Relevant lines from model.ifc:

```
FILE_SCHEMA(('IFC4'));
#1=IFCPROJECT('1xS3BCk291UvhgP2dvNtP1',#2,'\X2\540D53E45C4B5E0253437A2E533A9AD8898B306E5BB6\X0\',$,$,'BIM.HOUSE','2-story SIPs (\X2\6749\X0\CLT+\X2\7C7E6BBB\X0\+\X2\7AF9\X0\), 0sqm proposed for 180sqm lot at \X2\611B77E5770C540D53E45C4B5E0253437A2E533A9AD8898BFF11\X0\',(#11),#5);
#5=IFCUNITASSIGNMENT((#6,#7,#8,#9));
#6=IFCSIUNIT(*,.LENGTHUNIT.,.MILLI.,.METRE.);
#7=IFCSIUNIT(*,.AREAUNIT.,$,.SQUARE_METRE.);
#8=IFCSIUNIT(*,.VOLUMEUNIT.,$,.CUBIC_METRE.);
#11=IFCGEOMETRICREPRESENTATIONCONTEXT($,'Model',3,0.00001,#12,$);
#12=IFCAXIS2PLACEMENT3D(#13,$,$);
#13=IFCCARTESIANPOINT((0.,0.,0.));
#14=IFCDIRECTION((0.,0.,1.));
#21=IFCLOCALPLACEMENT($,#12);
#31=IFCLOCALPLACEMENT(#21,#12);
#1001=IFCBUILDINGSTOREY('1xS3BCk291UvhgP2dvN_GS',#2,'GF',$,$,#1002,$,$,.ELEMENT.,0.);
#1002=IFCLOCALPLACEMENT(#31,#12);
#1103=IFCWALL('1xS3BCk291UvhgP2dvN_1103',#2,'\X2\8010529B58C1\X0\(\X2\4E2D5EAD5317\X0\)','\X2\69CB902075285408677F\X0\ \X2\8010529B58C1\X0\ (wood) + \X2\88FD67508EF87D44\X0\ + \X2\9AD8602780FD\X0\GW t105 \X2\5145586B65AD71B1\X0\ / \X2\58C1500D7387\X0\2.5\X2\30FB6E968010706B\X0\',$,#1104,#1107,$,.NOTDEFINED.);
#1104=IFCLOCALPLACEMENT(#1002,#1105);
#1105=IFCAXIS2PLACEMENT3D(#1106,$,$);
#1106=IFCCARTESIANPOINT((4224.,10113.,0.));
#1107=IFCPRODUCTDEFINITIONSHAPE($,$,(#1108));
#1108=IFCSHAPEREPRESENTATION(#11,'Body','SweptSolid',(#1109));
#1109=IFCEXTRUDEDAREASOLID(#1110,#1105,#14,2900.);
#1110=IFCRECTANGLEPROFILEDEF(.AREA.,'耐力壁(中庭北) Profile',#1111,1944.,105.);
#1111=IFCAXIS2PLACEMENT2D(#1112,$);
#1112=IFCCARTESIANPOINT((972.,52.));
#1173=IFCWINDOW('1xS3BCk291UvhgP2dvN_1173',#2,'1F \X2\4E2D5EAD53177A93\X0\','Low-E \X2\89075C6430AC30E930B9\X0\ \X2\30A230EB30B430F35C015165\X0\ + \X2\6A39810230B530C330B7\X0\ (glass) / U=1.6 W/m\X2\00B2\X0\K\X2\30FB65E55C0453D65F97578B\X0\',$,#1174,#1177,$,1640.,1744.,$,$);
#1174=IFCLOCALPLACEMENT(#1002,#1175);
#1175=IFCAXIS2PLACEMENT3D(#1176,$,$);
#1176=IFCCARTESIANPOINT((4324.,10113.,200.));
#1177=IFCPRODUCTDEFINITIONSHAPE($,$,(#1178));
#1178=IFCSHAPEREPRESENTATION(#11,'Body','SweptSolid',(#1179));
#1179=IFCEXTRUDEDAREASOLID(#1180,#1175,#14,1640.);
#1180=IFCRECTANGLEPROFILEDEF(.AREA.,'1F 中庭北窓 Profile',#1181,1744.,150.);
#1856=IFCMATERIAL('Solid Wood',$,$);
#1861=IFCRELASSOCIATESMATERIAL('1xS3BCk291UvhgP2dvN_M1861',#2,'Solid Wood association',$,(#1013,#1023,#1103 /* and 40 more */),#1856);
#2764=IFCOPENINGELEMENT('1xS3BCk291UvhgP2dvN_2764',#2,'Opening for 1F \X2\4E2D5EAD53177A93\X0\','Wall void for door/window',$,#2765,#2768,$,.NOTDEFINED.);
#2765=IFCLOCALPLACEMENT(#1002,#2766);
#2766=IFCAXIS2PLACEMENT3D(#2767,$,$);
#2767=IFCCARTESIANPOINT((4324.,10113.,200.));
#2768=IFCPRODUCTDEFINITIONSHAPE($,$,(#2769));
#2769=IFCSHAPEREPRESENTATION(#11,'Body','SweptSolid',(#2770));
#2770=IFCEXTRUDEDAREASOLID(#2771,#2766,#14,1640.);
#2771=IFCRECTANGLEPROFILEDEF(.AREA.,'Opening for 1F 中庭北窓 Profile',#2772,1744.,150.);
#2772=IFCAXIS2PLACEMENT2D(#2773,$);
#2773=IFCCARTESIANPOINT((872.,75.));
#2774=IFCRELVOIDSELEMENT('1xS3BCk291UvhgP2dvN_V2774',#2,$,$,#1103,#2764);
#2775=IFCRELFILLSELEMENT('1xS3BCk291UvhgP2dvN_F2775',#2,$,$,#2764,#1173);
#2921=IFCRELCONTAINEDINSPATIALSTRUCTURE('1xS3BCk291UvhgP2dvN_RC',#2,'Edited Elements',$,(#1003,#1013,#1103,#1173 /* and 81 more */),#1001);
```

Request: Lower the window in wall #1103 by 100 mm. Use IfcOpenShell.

```python
import numpy as np
import ifcopenshell
import ifcopenshell.api.geometry
import ifcopenshell.util.placement
import ifcopenshell.util.unit

model = ifcopenshell.open("model.ifc")
unit_scale = ifcopenshell.util.unit.calculate_unit_scale(model)

window = model.by_id(1173)
opening = window.FillsVoids[0].RelatingOpeningElement
dz = -100.0

shift = np.array([0.0, 0.0, dz])
# The window is not placed relative to its opening, so move both.
for product in (opening, window):
    matrix = ifcopenshell.util.placement.get_local_placement(product.ObjectPlacement)
    matrix[:3, 3] += shift
    ifcopenshell.api.geometry.edit_object_placement(model, product=product, matrix=matrix, is_si=False)

print(f"moved by {dz * unit_scale:+.3f} m")

model.write("model_v2.ifc")
```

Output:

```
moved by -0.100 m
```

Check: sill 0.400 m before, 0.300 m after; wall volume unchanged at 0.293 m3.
